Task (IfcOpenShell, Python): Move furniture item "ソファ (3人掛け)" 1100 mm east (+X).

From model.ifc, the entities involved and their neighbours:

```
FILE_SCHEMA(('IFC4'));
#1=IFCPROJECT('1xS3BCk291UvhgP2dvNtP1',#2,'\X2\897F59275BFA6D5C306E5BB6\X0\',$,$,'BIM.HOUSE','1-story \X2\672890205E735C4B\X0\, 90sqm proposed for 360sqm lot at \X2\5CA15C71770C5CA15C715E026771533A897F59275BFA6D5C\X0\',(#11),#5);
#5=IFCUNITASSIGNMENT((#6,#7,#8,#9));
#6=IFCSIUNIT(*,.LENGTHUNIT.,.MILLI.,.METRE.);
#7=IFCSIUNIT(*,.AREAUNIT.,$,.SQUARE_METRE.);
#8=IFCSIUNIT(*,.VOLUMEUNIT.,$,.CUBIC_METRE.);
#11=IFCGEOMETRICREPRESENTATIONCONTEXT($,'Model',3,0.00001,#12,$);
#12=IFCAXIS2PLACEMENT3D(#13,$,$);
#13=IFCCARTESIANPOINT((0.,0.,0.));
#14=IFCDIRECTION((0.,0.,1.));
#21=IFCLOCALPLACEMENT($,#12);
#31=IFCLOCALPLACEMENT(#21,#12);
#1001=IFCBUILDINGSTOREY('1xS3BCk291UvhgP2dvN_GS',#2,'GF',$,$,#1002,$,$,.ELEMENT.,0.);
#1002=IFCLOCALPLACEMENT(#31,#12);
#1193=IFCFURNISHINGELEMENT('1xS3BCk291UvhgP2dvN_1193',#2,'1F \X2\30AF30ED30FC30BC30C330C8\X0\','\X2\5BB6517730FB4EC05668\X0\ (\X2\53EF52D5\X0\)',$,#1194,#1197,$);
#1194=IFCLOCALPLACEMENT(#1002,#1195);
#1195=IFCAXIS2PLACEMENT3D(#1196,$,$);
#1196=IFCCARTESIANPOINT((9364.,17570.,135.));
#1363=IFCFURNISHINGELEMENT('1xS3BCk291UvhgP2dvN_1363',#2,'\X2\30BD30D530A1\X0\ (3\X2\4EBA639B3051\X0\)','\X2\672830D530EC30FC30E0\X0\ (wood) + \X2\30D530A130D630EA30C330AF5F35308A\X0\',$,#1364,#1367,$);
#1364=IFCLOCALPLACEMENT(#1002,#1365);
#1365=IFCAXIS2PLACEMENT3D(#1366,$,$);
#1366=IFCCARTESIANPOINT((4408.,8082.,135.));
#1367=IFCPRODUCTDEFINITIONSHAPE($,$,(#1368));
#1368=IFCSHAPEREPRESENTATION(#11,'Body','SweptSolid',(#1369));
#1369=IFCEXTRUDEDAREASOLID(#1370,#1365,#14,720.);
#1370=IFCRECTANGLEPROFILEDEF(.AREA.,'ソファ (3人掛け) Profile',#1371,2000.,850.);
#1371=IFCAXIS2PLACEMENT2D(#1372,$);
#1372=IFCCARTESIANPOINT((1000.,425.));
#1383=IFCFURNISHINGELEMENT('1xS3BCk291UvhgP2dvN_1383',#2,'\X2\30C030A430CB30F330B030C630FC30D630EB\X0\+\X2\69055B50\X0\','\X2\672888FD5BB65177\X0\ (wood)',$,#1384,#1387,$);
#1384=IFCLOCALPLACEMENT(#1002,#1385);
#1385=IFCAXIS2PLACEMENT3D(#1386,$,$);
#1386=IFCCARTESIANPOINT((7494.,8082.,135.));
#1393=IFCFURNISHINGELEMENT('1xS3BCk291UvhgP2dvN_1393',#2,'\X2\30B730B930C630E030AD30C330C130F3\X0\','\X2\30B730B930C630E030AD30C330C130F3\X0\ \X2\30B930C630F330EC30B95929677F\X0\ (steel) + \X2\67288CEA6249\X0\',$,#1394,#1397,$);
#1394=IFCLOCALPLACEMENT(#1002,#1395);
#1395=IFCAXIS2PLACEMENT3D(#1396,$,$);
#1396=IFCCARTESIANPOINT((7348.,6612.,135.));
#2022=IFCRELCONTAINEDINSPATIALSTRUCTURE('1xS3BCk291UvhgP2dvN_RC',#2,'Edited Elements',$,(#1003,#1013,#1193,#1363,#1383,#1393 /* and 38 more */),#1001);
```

```python
import ifcopenshell
import ifcopenshell.api.geometry
import ifcopenshell.util.placement

model = ifcopenshell.open("model.ifc")

item = model.by_id(1363)
matrix = ifcopenshell.util.placement.get_local_placement(item.ObjectPlacement)
matrix[0, 3] += 1100.0
ifcopenshell.api.geometry.edit_object_placement(model, product=item, matrix=matrix, is_si=False)

print(ifcopenshell.util.placement.get_local_placement(item.ObjectPlacement).round(3) + 0.0)

model.write("model-out.ifc")
```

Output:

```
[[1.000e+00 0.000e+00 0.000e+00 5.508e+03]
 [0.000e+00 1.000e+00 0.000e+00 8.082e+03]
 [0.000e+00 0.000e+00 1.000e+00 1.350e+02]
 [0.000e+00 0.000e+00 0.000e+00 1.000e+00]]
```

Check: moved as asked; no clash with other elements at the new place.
